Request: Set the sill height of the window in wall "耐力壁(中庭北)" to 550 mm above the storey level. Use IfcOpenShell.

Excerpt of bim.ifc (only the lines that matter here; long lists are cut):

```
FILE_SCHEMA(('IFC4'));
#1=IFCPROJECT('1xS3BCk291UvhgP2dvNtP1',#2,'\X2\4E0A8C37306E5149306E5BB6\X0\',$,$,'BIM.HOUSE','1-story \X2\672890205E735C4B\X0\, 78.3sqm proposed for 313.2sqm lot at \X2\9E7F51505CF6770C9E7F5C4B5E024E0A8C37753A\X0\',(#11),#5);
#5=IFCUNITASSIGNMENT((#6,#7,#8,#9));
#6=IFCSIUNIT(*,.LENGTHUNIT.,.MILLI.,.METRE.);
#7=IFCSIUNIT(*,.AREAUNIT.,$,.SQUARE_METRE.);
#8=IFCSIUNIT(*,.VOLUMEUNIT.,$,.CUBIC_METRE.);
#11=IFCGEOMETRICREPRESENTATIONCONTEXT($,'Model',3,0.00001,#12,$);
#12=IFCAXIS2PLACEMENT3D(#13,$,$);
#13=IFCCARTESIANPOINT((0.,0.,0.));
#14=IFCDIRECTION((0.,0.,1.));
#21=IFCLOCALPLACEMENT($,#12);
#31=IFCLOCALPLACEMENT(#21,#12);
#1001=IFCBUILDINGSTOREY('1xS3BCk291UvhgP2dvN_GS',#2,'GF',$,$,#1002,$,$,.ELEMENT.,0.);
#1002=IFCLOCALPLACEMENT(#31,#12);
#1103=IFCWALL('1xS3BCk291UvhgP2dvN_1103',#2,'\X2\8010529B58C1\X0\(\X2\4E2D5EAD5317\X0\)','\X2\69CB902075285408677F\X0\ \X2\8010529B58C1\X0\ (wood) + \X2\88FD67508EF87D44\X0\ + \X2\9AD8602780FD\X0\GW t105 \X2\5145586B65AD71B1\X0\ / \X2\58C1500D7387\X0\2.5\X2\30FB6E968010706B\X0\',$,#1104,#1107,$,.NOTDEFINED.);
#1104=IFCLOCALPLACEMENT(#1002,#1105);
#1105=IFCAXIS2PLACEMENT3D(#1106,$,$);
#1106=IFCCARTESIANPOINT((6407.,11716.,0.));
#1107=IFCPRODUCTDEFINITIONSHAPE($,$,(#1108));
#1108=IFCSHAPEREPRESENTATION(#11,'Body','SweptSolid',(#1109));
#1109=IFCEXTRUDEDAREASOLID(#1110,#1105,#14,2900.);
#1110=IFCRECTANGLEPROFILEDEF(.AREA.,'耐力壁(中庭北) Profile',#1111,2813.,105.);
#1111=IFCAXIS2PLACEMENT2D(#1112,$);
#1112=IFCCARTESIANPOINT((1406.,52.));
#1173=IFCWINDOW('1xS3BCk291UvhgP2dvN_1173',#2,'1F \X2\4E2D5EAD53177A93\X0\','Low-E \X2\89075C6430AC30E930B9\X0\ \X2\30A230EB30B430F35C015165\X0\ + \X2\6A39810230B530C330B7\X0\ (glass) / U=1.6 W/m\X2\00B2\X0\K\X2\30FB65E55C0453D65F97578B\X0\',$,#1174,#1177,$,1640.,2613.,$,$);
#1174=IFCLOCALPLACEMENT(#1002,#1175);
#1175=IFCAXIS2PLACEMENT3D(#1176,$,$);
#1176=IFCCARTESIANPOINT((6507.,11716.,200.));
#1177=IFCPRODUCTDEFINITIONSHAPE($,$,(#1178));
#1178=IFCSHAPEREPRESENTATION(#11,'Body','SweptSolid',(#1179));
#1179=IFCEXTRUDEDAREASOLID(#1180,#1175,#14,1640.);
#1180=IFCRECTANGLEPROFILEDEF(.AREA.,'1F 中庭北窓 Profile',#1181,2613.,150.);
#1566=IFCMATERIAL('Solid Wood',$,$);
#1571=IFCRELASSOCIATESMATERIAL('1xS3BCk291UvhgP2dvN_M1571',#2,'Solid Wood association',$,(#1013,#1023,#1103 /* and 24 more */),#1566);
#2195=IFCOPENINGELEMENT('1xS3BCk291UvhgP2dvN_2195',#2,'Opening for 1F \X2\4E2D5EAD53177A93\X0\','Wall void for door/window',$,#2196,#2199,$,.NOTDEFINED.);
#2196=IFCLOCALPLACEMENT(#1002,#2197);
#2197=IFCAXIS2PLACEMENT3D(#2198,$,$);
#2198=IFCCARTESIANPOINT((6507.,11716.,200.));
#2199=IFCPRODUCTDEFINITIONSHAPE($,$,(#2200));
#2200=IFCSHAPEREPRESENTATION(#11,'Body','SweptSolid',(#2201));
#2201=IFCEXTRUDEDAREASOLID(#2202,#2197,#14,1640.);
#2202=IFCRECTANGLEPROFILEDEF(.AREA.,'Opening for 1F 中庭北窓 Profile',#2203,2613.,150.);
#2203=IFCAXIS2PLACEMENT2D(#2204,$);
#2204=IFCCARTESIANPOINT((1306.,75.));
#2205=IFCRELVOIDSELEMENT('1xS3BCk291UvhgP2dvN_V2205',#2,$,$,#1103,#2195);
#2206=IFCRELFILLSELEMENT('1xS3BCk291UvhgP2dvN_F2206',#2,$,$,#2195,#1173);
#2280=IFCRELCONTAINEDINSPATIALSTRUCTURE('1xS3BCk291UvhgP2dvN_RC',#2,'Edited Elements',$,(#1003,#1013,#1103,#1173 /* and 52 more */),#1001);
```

```python
import numpy as np
import ifcopenshell
import ifcopenshell.api.geometry
import ifcopenshell.geom
import ifcopenshell.util.element
import ifcopenshell.util.placement
import ifcopenshell.util.shape
import ifcopenshell.util.unit

model = ifcopenshell.open("bim.ifc")
unit_scale = ifcopenshell.util.unit.calculate_unit_scale(model)

window = model.by_guid("1xS3BCk291UvhgP2dvN_1173")
opening = window.FillsVoids[0].RelatingOpeningElement
storey = ifcopenshell.util.element.get_container(window, ifc_class="IfcBuildingStorey")
level = ifcopenshell.util.placement.get_local_placement(storey.ObjectPlacement)[2, 3]

# The opening's origin need not be at the sill, so measure its lowest point.
shape = ifcopenshell.geom.create_shape(ifcopenshell.geom.settings(), opening)
bottom = ifcopenshell.util.shape.get_shape_bottom_elevation(shape, shape.geometry) / unit_scale
dz = level + 550.0 - bottom

shift = np.array([0.0, 0.0, dz])
# The window is not placed relative to its opening, so move both.
for product in (opening, window):
    matrix = ifcopenshell.util.placement.get_local_placement(product.ObjectPlacement)
    matrix[:3, 3] += shift
    ifcopenshell.api.geometry.edit_object_placement(model, product=product, matrix=matrix, is_si=False)

print(f"moved by {dz * unit_scale:+.3f} m")

model.write("bim_updated.ifc")
```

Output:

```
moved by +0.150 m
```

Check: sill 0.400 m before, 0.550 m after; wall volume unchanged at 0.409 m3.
